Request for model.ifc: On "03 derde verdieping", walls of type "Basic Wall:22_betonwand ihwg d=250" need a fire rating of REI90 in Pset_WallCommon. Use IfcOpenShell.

First a look at what the model holds.

```python
import ifcopenshell
import ifcopenshell.util.element

model = ifcopenshell.open("model.ifc")
print(model.schema)
storey = next(s for s in model.by_type("IfcBuildingStorey") if s.Name == "03 derde verdieping")
walls = [e for e in ifcopenshell.util.element.get_decomposition(storey) if e.is_a("IfcWall")]
seen = {}
for e in walls:
    element_type = ifcopenshell.util.element.get_type(e)
    key = (element_type.Name if element_type != e and element_type else None, ifcopenshell.util.element.get_pset(e, "Pset_WallCommon", "FireRating"))
    seen[key] = seen.get(key, 0) + 1
for (name, value), count in sorted(seen.items(), key=str):
    print(count, "x", name, "|", value)
```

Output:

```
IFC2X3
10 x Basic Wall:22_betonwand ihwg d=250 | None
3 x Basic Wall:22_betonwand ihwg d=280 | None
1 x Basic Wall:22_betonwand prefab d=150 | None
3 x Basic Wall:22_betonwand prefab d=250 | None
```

```python
import ifcopenshell
import ifcopenshell.api.pset
import ifcopenshell.util.element

model = ifcopenshell.open("model.ifc")

storey = next(s for s in model.by_type("IfcBuildingStorey") if s.Name == "03 derde verdieping")
walls = [e for e in ifcopenshell.util.element.get_decomposition(storey) if e.is_a("IfcWall")]

count = 0
for e in walls:
    element_type = ifcopenshell.util.element.get_type(e)
    if element_type in (None, e) or element_type.Name != "Basic Wall:22_betonwand ihwg d=250":
        continue
    # add_pset returns the element's existing set when there is one.
    pset = ifcopenshell.api.pset.add_pset(model, product=e, name="Pset_WallCommon")
    ifcopenshell.api.pset.edit_pset(model, pset=pset, properties={"FireRating": "REI90"})
    count += 1

print(count, "walls updated")

model.write("model_rev.ifc")
```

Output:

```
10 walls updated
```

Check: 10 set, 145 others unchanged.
